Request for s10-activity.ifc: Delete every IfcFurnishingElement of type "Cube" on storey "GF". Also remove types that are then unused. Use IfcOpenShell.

First a look at what the model holds.

```python
import ifcopenshell
import ifcopenshell.util.element

model = ifcopenshell.open("s10-activity.ifc")
print(model.schema)
storey = next(s for s in model.by_type("IfcBuildingStorey") if s.Name == "GF")
furniture = [e for e in ifcopenshell.util.element.get_decomposition(storey) if e.is_a("IfcFurnishingElement")]
seen = {}
for e in furniture:
    element_type = ifcopenshell.util.element.get_type(e)
    name = element_type.Name if element_type not in (None, e) else None
    seen[name] = seen.get(name, 0) + 1
for name, count in sorted(seen.items(), key=str):
    print(count, "x", name)
```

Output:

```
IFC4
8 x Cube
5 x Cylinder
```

```python
import ifcopenshell
import ifcopenshell.api.root
import ifcopenshell.util.element

model = ifcopenshell.open("s10-activity.ifc")

storey = next(s for s in model.by_type("IfcBuildingStorey") if s.Name == "GF")
furniture = [e for e in ifcopenshell.util.element.get_decomposition(storey) if e.is_a("IfcFurnishingElement")]
targets = [e for e in furniture if (t := ifcopenshell.util.element.get_type(e)) not in (None, e) and t.Name == "Cube"]
types = {ifcopenshell.util.element.get_type(e) for e in targets} - {None, *targets}

for e in targets:
    ifcopenshell.api.root.remove_product(model, product=e)
print(len(targets), "removed")

unused = [t for t in types if not ifcopenshell.util.element.get_types(t)]
for t in unused:
    ifcopenshell.api.root.remove_product(model, product=t)
print(len(unused), "unused types removed")

model.write("s10-activity_rev.ifc")
```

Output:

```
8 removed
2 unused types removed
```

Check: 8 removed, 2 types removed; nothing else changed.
